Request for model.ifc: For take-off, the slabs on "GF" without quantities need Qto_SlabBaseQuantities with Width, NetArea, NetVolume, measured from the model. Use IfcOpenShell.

First a look at what the model holds.

```python
import ifcopenshell
import ifcopenshell.util.element
import ifcopenshell.util.unit

model = ifcopenshell.open("model.ifc")
print(model.schema)
for unit_type in ("LENGTHUNIT", "AREAUNIT", "VOLUMEUNIT"):
    print(unit_type, ifcopenshell.util.unit.calculate_unit_scale(model, unit_type))
storey = next(s for s in model.by_type("IfcBuildingStorey") if s.Name == "GF")
slabs = [e for e in ifcopenshell.util.element.get_decomposition(storey) if e.is_a("IfcSlab")]
for e in sorted(slabs, key=lambda e: e.id()):
    print(e.id(), e.is_a(), e.Name, list(ifcopenshell.util.element.get_psets(e, qtos_only=True)), sep=" | ")
```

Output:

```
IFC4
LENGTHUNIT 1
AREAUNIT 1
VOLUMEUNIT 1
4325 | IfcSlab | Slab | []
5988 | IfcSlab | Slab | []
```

```python
import ifcopenshell
import ifcopenshell.api.pset
import ifcopenshell.geom
import ifcopenshell.util.element
import ifcopenshell.util.shape
import ifcopenshell.util.unit

model = ifcopenshell.open("model.ifc")
unit_scale = ifcopenshell.util.unit.calculate_unit_scale(model)
area_scale = ifcopenshell.util.unit.calculate_unit_scale(model, "AREAUNIT")
volume_scale = ifcopenshell.util.unit.calculate_unit_scale(model, "VOLUMEUNIT")
settings = ifcopenshell.geom.settings()

storey = next(s for s in model.by_type("IfcBuildingStorey") if s.Name == "GF")
slabs = [e for e in ifcopenshell.util.element.get_decomposition(storey) if e.is_a("IfcSlab")]

for e in sorted(slabs, key=lambda e: e.id()):
    if ifcopenshell.util.element.get_psets(e, qtos_only=True, should_inherit=False):
        continue
    # Geometry comes back in metres, in the element's own axes.
    shape = ifcopenshell.geom.create_shape(settings, e)
    values = {
        "Width": ifcopenshell.util.shape.get_z(shape.geometry) / unit_scale,
        "NetArea": ifcopenshell.util.shape.get_footprint_area(shape.geometry) / area_scale,
        "NetVolume": ifcopenshell.util.shape.get_volume(shape.geometry) / volume_scale,
    }
    qto = ifcopenshell.api.pset.add_qto(model, product=e, name="Qto_SlabBaseQuantities")
    ifcopenshell.api.pset.edit_qto(model, qto=qto, properties=values)
    print(e.id(), {k: round(v, 3) for k, v in values.items()})

model.write("model-out.ifc")
```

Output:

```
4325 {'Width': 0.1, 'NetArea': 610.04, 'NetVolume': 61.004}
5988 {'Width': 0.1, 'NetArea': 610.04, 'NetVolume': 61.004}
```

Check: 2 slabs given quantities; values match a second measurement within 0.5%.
